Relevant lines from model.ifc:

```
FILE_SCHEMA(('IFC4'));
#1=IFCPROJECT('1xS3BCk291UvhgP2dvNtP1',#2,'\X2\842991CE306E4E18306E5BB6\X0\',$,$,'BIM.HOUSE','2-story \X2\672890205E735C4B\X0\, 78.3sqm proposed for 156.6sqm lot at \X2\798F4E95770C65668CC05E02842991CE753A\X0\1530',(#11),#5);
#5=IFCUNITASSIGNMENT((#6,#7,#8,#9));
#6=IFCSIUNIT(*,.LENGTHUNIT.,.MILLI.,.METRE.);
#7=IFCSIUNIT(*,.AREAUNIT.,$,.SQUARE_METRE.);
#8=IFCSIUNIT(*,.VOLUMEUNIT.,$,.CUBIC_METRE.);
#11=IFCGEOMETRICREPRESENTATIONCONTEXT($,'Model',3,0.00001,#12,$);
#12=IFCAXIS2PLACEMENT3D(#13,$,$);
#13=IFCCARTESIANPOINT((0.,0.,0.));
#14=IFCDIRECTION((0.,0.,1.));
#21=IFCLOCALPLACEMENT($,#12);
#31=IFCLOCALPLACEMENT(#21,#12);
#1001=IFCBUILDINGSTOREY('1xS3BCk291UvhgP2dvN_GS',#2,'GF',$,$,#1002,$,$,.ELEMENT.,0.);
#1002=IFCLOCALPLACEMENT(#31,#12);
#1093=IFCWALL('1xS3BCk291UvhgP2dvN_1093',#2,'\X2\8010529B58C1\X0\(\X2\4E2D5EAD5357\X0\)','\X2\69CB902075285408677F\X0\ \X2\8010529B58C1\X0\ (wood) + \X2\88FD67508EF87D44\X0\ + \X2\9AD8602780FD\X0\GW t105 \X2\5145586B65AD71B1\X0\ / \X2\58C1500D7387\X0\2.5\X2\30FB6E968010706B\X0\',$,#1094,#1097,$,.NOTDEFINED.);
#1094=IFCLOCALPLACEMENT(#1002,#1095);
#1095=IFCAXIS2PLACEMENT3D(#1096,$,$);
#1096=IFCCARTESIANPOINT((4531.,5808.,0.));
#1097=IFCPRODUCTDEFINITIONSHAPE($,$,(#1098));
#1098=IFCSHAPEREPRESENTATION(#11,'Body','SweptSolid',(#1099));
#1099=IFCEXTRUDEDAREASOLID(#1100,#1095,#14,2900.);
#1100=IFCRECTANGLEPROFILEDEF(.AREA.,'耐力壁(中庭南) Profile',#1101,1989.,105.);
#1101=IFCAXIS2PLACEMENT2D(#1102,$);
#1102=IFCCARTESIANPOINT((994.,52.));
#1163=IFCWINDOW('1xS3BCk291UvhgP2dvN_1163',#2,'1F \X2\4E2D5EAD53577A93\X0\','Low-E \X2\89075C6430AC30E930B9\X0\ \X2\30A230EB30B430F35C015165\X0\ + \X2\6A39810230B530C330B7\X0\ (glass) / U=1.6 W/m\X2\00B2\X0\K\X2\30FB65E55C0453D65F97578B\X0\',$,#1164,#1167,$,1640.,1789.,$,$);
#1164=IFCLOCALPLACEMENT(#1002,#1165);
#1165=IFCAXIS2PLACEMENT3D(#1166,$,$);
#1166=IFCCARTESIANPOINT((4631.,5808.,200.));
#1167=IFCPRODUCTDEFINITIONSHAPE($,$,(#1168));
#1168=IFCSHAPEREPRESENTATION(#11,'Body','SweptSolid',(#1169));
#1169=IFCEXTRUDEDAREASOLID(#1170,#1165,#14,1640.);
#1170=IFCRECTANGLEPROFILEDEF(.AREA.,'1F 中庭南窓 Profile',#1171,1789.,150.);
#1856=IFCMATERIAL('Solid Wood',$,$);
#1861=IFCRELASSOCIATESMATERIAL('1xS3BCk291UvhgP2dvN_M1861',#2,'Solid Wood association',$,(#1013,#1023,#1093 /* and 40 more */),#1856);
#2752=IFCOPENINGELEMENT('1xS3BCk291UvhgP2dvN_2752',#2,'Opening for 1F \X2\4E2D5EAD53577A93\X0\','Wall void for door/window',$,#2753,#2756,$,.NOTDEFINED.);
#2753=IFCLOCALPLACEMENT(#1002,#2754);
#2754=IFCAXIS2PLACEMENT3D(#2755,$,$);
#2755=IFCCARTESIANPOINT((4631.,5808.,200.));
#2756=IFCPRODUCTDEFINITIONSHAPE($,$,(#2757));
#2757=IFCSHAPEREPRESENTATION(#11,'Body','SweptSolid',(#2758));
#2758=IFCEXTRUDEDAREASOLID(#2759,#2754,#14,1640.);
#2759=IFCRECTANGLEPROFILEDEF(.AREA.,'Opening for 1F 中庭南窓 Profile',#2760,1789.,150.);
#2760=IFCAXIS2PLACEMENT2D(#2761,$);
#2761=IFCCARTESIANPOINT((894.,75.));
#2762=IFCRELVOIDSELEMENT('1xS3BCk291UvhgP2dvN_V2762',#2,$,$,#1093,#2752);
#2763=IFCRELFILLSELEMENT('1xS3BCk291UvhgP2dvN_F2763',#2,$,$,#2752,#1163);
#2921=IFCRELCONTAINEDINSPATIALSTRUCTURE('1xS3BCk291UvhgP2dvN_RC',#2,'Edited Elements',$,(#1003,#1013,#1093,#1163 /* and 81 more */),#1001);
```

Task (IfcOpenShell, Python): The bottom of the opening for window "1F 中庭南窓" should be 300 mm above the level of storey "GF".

```python
import numpy as np
import ifcopenshell
import ifcopenshell.api.geometry
import ifcopenshell.geom
import ifcopenshell.util.element
import ifcopenshell.util.placement
import ifcopenshell.util.shape
import ifcopenshell.util.unit

model = ifcopenshell.open("model.ifc")
unit_scale = ifcopenshell.util.unit.calculate_unit_scale(model)

window = model.by_guid("1xS3BCk291UvhgP2dvN_1163")
opening = window.FillsVoids[0].RelatingOpeningElement
storey = ifcopenshell.util.element.get_container(window, ifc_class="IfcBuildingStorey")
level = ifcopenshell.util.placement.get_local_placement(storey.ObjectPlacement)[2, 3]

# The opening's origin need not be at the sill, so measure its lowest point.
shape = ifcopenshell.geom.create_shape(ifcopenshell.geom.settings(), opening)
bottom = ifcopenshell.util.shape.get_shape_bottom_elevation(shape, shape.geometry) / unit_scale
dz = level + 0.3 / unit_scale - bottom

shift = np.array([0.0, 0.0, dz])
# The window is not placed relative to its opening, so move both.
for product in (opening, window):
    matrix = ifcopenshell.util.placement.get_local_placement(product.ObjectPlacement)
    matrix[:3, 3] += shift
    ifcopenshell.api.geometry.edit_object_placement(model, product=product, matrix=matrix, is_si=False)

print(f"moved by {dz * unit_scale:+.3f} m")

model.write("model_v2.ifc")
```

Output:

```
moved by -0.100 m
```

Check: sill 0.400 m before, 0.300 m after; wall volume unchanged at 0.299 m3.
